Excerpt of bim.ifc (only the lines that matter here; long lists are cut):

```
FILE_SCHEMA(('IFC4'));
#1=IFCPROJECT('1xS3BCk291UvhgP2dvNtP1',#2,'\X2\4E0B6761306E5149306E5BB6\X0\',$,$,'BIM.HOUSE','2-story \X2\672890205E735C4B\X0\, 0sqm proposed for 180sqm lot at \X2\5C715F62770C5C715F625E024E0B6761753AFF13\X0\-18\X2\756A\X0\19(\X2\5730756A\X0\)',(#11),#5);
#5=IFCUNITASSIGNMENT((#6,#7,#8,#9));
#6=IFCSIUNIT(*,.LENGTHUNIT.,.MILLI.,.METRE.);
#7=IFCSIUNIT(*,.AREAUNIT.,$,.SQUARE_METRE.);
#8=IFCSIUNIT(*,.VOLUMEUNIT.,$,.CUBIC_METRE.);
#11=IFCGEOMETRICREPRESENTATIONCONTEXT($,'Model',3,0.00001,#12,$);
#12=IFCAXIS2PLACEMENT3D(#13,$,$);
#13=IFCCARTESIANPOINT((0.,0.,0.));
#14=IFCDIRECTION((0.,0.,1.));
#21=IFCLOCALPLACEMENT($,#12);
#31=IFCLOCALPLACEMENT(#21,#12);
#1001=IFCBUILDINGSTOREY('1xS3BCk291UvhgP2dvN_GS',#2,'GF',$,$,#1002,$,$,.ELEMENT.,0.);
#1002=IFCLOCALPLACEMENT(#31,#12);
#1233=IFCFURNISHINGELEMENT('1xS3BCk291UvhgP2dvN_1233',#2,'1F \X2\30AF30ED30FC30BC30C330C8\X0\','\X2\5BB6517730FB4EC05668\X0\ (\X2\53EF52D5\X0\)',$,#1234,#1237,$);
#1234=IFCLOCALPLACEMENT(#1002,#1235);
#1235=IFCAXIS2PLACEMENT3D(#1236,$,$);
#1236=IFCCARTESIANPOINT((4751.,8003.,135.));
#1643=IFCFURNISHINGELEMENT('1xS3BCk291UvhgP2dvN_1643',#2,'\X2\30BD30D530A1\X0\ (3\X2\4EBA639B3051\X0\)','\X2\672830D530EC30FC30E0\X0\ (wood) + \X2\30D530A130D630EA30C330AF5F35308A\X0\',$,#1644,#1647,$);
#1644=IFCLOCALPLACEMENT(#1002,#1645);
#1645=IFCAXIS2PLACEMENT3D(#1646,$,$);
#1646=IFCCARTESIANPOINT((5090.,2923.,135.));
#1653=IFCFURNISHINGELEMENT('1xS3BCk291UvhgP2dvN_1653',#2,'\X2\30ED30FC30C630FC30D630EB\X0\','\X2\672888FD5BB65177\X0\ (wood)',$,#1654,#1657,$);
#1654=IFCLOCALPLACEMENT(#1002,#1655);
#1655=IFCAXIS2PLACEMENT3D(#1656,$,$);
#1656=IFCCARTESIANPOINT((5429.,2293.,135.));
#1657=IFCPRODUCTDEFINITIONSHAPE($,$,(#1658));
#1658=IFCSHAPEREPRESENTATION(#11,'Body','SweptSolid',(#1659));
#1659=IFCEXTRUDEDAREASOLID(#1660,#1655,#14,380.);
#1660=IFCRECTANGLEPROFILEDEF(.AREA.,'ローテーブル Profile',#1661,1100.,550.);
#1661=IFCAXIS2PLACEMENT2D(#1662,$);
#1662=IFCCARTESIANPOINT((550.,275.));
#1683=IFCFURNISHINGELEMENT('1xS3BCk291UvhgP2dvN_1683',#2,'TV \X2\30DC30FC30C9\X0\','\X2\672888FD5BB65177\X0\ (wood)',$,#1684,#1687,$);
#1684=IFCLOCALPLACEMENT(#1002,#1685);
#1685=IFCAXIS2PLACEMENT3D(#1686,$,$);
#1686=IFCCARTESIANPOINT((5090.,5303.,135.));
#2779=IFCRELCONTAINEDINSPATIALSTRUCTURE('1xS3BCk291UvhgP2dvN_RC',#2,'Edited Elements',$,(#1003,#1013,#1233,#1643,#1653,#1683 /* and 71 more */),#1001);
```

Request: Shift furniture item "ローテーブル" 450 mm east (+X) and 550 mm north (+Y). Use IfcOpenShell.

```python
import ifcopenshell
import ifcopenshell.api.geometry
import ifcopenshell.util.placement

model = ifcopenshell.open("bim.ifc")

item = model.by_id(1653)
matrix = ifcopenshell.util.placement.get_local_placement(item.ObjectPlacement)
matrix[0, 3] += 450.0
matrix[1, 3] += 550.0
ifcopenshell.api.geometry.edit_object_placement(model, product=item, matrix=matrix, is_si=False)

print(ifcopenshell.util.placement.get_local_placement(item.ObjectPlacement).round(3) + 0.0)

model.write("bim_edited.ifc")
```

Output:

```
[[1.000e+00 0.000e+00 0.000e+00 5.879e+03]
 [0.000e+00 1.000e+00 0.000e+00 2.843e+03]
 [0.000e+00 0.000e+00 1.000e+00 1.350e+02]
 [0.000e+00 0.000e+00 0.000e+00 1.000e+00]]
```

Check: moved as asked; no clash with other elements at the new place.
